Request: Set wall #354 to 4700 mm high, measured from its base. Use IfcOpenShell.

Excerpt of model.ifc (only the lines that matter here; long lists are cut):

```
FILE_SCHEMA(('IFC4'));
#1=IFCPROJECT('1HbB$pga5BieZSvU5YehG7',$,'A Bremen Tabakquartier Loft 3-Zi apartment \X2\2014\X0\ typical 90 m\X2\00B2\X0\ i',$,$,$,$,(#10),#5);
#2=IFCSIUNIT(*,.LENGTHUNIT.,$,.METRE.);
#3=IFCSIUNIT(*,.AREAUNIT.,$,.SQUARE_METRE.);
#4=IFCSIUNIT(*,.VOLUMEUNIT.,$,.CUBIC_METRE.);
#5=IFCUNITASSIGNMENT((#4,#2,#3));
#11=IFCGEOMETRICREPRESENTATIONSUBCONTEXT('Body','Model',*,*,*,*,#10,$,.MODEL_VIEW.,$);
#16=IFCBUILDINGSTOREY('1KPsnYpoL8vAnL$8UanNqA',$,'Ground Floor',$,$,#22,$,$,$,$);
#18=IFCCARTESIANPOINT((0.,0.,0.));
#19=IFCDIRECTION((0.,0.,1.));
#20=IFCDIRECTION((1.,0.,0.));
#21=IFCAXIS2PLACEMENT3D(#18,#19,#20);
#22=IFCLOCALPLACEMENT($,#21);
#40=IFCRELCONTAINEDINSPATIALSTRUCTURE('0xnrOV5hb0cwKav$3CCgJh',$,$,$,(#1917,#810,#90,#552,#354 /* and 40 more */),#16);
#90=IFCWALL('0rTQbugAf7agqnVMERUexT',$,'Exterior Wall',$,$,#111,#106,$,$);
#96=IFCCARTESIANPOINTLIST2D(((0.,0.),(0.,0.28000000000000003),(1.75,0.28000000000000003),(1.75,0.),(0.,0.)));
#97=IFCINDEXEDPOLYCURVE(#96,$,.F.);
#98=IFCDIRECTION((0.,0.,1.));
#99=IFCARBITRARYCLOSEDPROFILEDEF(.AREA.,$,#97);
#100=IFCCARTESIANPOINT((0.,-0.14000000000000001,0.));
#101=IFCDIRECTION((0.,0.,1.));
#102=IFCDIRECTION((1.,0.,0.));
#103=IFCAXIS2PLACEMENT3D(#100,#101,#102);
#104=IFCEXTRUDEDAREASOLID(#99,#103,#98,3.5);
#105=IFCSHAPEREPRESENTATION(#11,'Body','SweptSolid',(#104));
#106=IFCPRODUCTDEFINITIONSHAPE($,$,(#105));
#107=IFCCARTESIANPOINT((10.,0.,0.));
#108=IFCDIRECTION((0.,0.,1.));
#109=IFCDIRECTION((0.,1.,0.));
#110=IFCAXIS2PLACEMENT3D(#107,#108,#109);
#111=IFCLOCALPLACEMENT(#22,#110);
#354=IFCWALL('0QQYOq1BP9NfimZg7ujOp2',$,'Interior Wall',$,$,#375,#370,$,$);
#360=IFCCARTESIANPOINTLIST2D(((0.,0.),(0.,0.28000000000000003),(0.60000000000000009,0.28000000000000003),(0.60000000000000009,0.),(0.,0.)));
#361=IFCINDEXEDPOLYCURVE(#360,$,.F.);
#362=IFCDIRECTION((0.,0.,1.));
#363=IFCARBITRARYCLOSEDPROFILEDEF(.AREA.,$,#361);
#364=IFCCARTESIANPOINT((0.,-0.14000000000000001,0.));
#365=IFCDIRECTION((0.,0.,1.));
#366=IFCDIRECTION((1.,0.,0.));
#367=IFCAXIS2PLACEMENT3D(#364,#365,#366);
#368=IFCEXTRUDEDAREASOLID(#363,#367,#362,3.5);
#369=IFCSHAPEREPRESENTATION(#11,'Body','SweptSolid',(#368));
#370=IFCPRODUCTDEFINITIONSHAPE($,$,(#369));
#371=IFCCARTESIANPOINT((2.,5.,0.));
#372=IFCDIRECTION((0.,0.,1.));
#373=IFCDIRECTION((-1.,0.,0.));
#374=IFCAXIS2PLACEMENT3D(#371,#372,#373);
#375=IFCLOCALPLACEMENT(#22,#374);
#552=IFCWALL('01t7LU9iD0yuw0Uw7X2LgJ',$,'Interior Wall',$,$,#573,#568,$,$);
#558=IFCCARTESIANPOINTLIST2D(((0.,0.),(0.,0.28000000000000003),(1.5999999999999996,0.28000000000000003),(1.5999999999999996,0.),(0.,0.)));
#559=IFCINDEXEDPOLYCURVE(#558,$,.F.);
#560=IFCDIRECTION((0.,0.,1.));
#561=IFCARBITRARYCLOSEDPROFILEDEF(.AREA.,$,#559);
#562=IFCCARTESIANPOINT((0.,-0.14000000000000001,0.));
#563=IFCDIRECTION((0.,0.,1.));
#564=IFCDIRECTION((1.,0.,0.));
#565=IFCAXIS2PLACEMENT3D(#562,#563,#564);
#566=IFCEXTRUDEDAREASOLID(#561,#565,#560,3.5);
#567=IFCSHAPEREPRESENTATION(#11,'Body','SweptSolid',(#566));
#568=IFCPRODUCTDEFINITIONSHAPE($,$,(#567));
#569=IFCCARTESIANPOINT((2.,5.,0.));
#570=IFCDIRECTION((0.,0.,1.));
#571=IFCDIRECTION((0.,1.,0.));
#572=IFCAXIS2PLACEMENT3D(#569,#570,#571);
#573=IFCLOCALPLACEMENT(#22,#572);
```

```python
import ifcopenshell
import ifcopenshell.geom
import ifcopenshell.util.representation
import ifcopenshell.util.shape
import ifcopenshell.util.unit

model = ifcopenshell.open("model.ifc")
unit_scale = ifcopenshell.util.unit.calculate_unit_scale(model)
settings = ifcopenshell.geom.settings()


def volume(element):
    """Net volume in cubic metres, openings subtracted."""
    shape = ifcopenshell.geom.create_shape(settings, element)
    return ifcopenshell.util.shape.get_volume(shape.geometry)


wall = model.by_guid("0QQYOq1BP9NfimZg7ujOp2")
before = volume(wall)

body = ifcopenshell.util.representation.get_representation(wall, "Model", "Body")
solid = body.Items[0]
old_height = solid.Depth
solid.Depth = 4.7 / unit_scale
after = volume(wall)

print(f"height {old_height:g} -> {solid.Depth:g}, volume {before:.3f} -> {after:.3f} m3")

model.write("model_v2.ifc")
```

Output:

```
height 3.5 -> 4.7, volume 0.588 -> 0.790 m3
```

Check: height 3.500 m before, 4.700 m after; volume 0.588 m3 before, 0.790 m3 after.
